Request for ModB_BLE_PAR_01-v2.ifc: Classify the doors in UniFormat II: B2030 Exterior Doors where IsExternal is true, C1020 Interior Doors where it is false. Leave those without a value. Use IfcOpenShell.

First a look at what the model holds.

```python
import ifcopenshell
import ifcopenshell.util.element

model = ifcopenshell.open("ModB_BLE_PAR_01-v2.ifc")
print(model.schema)
print("classifications:", [c.Name for c in model.by_type("IfcClassification")])
values = [ifcopenshell.util.element.get_pset(e, "Pset_DoorCommon", "IsExternal") for e in model.by_type("IfcDoor")]
for value in (True, False, None):
    print("IsExternal", value, values.count(value))
```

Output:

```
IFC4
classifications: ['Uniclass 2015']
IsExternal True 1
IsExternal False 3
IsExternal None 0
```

```python
import ifcopenshell
import ifcopenshell.api.classification
import ifcopenshell.util.element

model = ifcopenshell.open("ModB_BLE_PAR_01-v2.ifc")

system = ifcopenshell.api.classification.add_classification(model, classification="UniFormat II")

doors = model.by_type("IfcDoor")
external = {e: ifcopenshell.util.element.get_pset(e, "Pset_DoorCommon", "IsExternal") for e in doors}
for flag, code, name in ((True, "B2030", "Exterior Doors"), (False, "C1020", "Interior Doors")):
    products = [e for e in doors if external[e] is flag]
    ifcopenshell.api.classification.add_reference(
        model, products=products, classification=system, identification=code, name=name
    )
    print(code, len(products))

model.write("ModB_BLE_PAR_01-v2-out.ifc")
```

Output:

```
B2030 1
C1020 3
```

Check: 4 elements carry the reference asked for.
